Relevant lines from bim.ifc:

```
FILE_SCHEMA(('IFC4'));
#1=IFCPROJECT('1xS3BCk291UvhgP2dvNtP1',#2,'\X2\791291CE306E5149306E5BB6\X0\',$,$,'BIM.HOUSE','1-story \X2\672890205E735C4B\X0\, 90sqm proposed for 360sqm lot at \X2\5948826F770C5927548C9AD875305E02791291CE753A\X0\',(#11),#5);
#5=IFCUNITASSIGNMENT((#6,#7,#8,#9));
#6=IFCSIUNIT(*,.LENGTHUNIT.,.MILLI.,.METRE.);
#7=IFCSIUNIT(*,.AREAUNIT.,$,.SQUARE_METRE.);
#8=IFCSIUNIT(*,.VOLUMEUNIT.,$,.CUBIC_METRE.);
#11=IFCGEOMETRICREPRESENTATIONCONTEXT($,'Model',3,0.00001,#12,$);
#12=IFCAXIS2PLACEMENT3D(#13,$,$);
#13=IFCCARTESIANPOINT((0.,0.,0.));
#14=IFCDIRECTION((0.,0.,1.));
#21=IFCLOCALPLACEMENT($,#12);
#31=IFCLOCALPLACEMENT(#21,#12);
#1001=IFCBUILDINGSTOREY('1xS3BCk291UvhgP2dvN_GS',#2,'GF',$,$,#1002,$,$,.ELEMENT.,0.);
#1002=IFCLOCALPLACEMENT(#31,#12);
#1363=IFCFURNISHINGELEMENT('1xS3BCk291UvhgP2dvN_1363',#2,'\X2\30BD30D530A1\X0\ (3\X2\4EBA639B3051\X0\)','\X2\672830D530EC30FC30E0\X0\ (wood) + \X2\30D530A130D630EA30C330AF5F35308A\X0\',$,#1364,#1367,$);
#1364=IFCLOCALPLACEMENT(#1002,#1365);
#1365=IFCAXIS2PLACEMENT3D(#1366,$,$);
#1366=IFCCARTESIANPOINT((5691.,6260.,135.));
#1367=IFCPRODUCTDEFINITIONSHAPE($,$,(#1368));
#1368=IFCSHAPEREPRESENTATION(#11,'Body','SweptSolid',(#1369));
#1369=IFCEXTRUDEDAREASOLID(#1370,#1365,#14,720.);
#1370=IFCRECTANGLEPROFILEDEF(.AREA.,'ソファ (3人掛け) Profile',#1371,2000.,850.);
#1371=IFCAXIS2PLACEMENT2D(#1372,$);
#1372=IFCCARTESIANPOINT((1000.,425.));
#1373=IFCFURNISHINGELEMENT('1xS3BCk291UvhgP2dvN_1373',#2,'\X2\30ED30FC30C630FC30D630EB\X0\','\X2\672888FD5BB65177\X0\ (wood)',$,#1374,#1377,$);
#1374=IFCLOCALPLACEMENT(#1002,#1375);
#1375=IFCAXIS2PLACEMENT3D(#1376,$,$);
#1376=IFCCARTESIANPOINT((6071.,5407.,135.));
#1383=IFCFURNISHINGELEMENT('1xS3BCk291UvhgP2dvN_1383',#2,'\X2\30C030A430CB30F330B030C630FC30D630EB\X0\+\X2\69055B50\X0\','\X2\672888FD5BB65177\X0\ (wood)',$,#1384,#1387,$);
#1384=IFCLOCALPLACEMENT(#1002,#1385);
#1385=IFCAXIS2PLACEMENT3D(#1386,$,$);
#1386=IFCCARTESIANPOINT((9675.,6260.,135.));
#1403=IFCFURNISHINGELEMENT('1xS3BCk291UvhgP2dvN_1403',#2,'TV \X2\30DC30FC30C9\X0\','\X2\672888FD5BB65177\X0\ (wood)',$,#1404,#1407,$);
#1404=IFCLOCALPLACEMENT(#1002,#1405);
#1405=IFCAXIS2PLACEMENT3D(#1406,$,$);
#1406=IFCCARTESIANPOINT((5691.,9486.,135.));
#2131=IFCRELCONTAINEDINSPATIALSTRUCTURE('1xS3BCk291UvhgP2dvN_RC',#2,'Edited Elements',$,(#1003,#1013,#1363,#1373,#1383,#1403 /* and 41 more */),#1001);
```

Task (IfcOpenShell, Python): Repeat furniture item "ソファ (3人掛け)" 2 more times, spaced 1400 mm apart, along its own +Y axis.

```python
import ifcopenshell
import ifcopenshell.api.geometry
import ifcopenshell.api.root
import ifcopenshell.util.element
import ifcopenshell.util.placement
import ifcopenshell.util.unit

model = ifcopenshell.open("bim.ifc")
unit_scale = ifcopenshell.util.unit.calculate_unit_scale(model)


def reuse_history(source, copy):
    """copy_class also copies each property set's owner history, people and application; keep the originals."""
    for rel in copy.IsDefinedBy:
        if rel.is_a("IfcRelDefinesByProperties") and (history := rel.RelatingPropertyDefinition.OwnerHistory):
            rel.RelatingPropertyDefinition.OwnerHistory = source.OwnerHistory
            ifcopenshell.util.element.remove_deep2(model, history)


source = model.by_guid("1xS3BCk291UvhgP2dvN_1363")
base = ifcopenshell.util.placement.get_local_placement(source.ObjectPlacement)
step = base[:3, 1] * 1.4 / unit_scale

for i in range(1, 3):
    copy = ifcopenshell.api.root.copy_class(model, product=source)
    copy.Representation = ifcopenshell.util.element.copy_deep(
        model, source.Representation, exclude=["IfcGeometricRepresentationContext", "IfcRepresentationMap"]
    )
    reuse_history(source, copy)
    matrix = base.copy()
    matrix[:3, 3] += i * step
    print("added at", matrix[:3, 3].round(3) + 0.0)
    ifcopenshell.api.geometry.edit_object_placement(model, product=copy, matrix=matrix, is_si=False)

model.write("bim_updated.ifc")
```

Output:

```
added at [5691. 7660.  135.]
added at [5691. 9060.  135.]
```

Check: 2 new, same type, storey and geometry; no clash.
